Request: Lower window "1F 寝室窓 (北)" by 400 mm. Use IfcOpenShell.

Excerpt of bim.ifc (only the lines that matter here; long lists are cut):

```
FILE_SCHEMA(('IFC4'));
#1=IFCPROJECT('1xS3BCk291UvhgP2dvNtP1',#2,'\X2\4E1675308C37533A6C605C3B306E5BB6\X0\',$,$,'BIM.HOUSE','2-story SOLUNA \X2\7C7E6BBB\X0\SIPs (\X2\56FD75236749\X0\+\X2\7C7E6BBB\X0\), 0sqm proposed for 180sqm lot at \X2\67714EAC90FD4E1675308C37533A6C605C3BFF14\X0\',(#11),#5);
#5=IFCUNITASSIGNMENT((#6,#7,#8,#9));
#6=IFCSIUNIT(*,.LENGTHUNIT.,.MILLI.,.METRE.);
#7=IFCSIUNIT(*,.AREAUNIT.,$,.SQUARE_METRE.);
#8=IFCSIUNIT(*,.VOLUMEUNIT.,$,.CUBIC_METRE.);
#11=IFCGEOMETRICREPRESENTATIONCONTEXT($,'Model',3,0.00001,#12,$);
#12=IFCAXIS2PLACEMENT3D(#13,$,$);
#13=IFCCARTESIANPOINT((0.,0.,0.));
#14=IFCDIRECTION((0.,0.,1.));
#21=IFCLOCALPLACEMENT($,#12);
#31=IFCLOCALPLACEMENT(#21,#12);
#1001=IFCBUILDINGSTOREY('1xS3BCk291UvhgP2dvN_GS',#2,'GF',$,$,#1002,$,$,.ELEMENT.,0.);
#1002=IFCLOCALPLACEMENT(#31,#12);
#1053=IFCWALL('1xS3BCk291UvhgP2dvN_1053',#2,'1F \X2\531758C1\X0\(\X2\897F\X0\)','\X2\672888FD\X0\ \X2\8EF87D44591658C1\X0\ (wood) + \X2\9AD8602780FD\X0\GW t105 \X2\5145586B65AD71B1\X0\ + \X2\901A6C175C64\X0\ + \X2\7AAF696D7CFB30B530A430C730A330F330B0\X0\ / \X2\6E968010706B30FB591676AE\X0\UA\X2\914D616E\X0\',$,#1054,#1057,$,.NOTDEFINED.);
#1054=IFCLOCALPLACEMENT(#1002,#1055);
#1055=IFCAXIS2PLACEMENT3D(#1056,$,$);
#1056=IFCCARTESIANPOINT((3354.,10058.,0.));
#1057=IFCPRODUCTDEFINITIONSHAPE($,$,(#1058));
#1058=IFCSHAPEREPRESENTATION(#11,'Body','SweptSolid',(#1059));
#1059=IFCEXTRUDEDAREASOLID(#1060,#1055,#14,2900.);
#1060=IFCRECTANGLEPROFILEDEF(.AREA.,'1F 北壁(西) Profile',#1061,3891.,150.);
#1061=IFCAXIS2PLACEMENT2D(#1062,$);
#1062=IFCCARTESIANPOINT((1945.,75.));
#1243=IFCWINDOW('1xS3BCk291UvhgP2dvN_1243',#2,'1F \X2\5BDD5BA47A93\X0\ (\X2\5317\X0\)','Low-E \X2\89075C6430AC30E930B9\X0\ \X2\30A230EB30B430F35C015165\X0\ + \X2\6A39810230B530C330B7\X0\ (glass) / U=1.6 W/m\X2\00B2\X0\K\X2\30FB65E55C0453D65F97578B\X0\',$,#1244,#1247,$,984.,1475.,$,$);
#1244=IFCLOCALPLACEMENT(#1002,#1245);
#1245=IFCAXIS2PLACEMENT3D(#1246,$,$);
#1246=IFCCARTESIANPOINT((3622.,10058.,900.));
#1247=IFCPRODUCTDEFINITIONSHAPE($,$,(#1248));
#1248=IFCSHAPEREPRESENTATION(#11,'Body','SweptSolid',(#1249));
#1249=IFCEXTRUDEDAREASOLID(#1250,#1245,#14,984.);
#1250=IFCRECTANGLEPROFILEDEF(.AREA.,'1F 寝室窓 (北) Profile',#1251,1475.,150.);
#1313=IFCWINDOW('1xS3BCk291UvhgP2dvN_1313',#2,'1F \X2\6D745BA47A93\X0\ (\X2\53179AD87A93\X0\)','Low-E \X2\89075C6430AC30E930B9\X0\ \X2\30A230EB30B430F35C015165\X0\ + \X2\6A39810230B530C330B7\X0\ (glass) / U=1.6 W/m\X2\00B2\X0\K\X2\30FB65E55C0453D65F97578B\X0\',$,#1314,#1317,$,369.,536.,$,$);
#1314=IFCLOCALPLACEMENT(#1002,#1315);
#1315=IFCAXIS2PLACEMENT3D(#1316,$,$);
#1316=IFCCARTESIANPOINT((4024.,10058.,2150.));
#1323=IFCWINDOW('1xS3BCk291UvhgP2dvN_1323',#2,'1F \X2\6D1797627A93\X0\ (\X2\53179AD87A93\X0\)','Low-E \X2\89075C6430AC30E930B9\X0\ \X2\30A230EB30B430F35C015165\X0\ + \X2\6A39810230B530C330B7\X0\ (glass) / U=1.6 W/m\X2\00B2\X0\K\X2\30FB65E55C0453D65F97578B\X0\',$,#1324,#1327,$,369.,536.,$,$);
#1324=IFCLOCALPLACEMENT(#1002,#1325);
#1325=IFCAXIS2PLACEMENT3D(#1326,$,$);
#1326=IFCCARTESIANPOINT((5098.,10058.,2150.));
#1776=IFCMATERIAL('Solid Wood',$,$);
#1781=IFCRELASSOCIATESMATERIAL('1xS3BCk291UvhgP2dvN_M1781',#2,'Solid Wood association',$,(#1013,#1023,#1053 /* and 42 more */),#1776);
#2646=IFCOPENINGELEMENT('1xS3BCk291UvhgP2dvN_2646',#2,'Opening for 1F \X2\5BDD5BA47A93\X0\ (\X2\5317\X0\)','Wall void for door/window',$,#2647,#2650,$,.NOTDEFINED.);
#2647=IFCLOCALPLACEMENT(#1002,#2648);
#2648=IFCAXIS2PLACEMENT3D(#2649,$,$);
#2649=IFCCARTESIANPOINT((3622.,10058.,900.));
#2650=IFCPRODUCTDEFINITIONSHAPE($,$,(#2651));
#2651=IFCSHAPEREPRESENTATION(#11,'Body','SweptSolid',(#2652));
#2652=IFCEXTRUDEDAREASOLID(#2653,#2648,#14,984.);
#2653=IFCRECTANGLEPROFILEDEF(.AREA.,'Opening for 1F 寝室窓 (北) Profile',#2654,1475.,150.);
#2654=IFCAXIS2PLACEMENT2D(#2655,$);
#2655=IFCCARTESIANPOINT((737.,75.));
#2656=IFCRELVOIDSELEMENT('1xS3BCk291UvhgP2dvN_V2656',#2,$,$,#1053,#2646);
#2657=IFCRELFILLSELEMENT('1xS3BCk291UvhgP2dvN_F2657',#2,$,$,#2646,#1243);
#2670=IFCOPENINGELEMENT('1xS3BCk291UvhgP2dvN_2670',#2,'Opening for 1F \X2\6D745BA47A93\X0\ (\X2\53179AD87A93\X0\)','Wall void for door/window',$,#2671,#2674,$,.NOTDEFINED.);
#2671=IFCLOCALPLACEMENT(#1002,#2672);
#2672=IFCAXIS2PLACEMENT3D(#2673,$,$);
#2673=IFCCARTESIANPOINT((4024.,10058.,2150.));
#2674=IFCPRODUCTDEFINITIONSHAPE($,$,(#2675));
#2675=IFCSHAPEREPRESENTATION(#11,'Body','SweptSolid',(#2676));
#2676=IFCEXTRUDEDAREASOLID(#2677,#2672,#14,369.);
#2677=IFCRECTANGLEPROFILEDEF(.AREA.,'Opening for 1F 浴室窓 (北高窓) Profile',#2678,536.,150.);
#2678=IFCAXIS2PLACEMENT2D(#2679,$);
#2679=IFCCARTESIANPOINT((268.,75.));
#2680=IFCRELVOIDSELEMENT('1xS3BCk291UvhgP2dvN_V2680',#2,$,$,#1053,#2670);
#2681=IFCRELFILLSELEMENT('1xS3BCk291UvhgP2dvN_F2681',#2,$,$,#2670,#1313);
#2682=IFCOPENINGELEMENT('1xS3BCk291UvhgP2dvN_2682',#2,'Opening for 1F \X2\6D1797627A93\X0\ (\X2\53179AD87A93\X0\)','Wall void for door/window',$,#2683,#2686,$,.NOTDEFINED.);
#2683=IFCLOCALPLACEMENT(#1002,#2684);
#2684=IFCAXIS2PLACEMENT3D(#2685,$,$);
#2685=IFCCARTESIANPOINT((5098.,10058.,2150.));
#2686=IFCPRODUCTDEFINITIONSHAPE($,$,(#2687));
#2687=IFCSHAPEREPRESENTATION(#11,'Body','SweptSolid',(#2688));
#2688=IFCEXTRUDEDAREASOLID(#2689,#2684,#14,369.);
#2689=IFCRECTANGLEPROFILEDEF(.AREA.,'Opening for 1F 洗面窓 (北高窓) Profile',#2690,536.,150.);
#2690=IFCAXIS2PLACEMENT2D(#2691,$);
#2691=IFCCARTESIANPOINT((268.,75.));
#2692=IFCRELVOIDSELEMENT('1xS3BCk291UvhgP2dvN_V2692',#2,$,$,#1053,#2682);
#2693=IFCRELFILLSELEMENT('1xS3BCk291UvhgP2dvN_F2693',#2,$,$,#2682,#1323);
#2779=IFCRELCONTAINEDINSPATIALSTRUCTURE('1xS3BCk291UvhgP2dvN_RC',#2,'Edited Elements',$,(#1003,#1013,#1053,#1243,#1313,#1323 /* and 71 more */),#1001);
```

```python
import numpy as np
import ifcopenshell
import ifcopenshell.api.geometry
import ifcopenshell.util.placement
import ifcopenshell.util.unit

model = ifcopenshell.open("bim.ifc")
unit_scale = ifcopenshell.util.unit.calculate_unit_scale(model)

window = model.by_guid("1xS3BCk291UvhgP2dvN_1243")
opening = window.FillsVoids[0].RelatingOpeningElement
dz = -0.4 / unit_scale

shift = np.array([0.0, 0.0, dz])
# The window is not placed relative to its opening, so move both.
for product in (opening, window):
    matrix = ifcopenshell.util.placement.get_local_placement(product.ObjectPlacement)
    matrix[:3, 3] += shift
    ifcopenshell.api.geometry.edit_object_placement(model, product=product, matrix=matrix, is_si=False)

print(f"moved by {dz * unit_scale:+.3f} m")

model.write("bim-out.ifc")
```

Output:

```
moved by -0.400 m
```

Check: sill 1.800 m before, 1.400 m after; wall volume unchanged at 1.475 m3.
